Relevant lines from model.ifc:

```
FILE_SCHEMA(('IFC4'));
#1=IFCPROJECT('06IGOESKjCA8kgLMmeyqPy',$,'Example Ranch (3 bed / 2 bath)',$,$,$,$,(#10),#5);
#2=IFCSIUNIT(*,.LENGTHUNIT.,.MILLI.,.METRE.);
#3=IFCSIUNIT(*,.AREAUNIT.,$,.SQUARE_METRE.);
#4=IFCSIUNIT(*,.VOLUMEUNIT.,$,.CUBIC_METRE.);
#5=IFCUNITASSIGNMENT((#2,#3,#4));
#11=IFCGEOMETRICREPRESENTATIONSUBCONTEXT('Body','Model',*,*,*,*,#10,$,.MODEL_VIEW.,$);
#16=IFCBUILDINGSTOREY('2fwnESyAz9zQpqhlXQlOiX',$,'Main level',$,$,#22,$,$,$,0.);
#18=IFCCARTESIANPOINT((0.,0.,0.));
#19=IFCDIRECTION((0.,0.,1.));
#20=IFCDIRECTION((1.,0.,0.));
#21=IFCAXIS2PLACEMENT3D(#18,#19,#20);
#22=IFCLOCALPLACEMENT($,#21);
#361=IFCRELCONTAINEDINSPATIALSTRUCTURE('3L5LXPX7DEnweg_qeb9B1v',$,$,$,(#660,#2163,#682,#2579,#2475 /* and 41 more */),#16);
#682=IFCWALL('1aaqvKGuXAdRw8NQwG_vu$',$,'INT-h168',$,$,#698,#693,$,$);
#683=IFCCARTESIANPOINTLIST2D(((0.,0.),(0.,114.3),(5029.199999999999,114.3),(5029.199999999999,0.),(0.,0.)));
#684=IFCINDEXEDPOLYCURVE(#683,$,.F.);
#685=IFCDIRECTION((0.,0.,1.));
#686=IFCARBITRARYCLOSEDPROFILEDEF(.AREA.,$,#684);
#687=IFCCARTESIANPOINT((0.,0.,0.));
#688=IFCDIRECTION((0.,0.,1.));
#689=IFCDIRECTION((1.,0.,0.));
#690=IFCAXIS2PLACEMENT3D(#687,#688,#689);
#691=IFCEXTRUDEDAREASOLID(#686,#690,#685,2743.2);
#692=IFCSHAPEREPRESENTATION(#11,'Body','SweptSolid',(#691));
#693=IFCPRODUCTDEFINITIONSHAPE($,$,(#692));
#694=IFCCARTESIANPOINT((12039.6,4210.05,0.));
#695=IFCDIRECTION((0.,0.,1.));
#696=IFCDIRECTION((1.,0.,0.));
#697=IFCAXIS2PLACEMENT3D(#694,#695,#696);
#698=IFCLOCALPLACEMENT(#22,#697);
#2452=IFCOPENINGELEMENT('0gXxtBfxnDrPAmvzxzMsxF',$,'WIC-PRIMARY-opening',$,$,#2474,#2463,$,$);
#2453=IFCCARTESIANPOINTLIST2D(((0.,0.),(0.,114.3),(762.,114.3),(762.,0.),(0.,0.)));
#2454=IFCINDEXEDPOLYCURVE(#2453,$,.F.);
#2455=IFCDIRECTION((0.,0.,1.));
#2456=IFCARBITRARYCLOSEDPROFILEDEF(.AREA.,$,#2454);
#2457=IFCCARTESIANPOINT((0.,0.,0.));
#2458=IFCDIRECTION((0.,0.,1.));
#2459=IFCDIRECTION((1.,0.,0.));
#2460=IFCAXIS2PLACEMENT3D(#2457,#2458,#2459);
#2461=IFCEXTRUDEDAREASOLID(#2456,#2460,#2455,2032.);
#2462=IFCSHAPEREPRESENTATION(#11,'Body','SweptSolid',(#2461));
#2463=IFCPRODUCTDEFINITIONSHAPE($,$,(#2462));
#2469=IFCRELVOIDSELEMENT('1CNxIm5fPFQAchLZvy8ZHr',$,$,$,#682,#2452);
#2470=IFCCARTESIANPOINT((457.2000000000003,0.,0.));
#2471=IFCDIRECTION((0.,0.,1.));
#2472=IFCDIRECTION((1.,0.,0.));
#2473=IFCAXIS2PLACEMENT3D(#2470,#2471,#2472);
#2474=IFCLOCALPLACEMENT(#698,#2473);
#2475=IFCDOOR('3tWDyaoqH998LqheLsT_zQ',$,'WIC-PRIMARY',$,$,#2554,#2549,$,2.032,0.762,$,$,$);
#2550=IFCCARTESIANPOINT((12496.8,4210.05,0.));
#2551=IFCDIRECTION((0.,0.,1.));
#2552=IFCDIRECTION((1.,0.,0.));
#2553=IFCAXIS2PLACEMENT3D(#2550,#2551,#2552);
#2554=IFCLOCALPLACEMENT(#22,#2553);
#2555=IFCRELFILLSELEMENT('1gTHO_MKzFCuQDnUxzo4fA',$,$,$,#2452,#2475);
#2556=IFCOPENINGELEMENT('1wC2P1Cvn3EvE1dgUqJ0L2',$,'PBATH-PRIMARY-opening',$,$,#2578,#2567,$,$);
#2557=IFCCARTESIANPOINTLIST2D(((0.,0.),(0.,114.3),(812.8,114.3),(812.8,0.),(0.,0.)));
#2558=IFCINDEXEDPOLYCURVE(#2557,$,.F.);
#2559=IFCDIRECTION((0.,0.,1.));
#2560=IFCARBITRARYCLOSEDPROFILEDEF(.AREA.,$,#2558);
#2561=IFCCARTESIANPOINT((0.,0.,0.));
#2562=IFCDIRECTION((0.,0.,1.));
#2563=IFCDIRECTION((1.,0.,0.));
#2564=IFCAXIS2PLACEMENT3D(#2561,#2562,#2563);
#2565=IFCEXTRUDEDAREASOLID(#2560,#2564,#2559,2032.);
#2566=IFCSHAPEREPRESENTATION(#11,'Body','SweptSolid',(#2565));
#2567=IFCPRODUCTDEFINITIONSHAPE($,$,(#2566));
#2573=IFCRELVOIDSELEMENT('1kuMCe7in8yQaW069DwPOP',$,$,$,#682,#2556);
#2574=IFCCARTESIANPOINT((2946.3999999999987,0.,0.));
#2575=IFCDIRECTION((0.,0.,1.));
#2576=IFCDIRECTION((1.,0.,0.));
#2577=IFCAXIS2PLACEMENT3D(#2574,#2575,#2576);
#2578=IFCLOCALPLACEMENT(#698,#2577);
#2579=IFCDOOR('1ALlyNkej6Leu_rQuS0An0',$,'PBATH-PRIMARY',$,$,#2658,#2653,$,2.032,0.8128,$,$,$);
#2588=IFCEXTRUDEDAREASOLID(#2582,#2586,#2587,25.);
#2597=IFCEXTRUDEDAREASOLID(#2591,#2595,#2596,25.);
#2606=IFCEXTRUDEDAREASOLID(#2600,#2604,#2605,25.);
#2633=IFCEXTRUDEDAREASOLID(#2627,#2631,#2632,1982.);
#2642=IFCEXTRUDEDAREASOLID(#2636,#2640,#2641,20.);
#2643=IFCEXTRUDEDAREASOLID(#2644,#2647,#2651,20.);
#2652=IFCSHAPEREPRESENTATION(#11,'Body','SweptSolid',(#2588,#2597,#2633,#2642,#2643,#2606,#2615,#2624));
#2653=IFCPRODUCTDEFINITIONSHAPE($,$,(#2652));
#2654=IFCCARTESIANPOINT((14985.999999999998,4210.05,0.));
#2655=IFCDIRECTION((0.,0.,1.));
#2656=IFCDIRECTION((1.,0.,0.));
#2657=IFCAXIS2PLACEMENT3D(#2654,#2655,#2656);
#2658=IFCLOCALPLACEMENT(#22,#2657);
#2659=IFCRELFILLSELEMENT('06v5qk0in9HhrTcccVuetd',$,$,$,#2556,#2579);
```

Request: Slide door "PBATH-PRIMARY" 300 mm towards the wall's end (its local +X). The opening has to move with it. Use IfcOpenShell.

```python
import ifcopenshell
import ifcopenshell.api.geometry
import ifcopenshell.util.placement
import ifcopenshell.util.unit

model = ifcopenshell.open("model.ifc")
unit_scale = ifcopenshell.util.unit.calculate_unit_scale(model)

door = model.by_id(2579)
opening = door.FillsVoids[0].RelatingOpeningElement
wall = opening.VoidsElements[0].RelatingBuildingElement

wall_matrix = ifcopenshell.util.placement.get_local_placement(wall.ObjectPlacement)
shift = wall_matrix[:3, 0] * 0.3 / unit_scale
before = ifcopenshell.util.placement.get_local_placement(door.ObjectPlacement)[:3, 3].copy()

# The door is not placed relative to its opening, so move both.
for product in (opening, door):
    matrix = ifcopenshell.util.placement.get_local_placement(product.ObjectPlacement)
    matrix[:3, 3] += shift
    ifcopenshell.api.geometry.edit_object_placement(model, product=product, matrix=matrix, is_si=False)

after = ifcopenshell.util.placement.get_local_placement(door.ObjectPlacement)[:3, 3]
print("door moved by", (after - before).round(3) + 0.0)

model.write("model_rev.ifc")
```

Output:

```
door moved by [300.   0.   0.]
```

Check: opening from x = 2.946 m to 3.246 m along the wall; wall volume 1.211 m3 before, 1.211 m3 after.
